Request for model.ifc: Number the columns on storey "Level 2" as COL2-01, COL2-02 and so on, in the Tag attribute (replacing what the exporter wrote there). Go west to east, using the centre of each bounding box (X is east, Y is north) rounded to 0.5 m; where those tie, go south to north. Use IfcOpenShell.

First a look at what the model holds.

```python
import ifcopenshell
import ifcopenshell.util.element
import ifcopenshell.util.placement

model = ifcopenshell.open("model.ifc")
print(model.schema)
storey = next(s for s in model.by_type("IfcBuildingStorey") if s.Name == "Level 2")
columns = [e for e in ifcopenshell.util.element.get_decomposition(storey) if e.is_a("IfcColumn")]
for e in sorted(columns, key=lambda e: e.id()):
    origin = ifcopenshell.util.placement.get_local_placement(e.ObjectPlacement)[:3, 3]
    print(e.id(), e.Tag, e.Name, origin.round(2) + 0.0, sep=" | ")
```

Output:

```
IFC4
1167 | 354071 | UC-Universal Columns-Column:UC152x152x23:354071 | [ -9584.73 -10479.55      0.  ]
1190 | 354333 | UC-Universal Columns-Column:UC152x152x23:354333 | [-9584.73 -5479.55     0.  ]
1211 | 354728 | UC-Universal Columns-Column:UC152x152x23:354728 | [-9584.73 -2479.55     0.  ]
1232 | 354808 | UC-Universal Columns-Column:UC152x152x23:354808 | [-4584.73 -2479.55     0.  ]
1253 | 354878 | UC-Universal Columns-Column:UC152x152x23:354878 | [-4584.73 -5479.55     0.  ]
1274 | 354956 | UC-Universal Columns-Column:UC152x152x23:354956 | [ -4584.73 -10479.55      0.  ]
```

```python
import ifcopenshell
import ifcopenshell.geom
import ifcopenshell.util.element
import ifcopenshell.util.shape

model = ifcopenshell.open("model.ifc")
settings = ifcopenshell.geom.settings()
settings.set("use-world-coords", True)


def centre(element):
    shape = ifcopenshell.geom.create_shape(settings, element)
    return ifcopenshell.util.shape.get_bbox_centroid(shape.geometry)


storey = next(s for s in model.by_type("IfcBuildingStorey") if s.Name == "Level 2")
columns = [e for e in ifcopenshell.util.element.get_decomposition(storey) if e.is_a("IfcColumn")]

# Insertion points can sit at a corner or the storey origin, so sort by the geometry (in metres).
centres = {e: centre(e) for e in columns}
columns.sort(key=lambda e: (round(centres[e][0] / 0.5), centres[e][1]))

for i, e in enumerate(columns, start=1):
    number = f"COL2-{i:02d}"
    e.Tag = number
    print(e.id(), number)

model.write("model_updated.ifc")
```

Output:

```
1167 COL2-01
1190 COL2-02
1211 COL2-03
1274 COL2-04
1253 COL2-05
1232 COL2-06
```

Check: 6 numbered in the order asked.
